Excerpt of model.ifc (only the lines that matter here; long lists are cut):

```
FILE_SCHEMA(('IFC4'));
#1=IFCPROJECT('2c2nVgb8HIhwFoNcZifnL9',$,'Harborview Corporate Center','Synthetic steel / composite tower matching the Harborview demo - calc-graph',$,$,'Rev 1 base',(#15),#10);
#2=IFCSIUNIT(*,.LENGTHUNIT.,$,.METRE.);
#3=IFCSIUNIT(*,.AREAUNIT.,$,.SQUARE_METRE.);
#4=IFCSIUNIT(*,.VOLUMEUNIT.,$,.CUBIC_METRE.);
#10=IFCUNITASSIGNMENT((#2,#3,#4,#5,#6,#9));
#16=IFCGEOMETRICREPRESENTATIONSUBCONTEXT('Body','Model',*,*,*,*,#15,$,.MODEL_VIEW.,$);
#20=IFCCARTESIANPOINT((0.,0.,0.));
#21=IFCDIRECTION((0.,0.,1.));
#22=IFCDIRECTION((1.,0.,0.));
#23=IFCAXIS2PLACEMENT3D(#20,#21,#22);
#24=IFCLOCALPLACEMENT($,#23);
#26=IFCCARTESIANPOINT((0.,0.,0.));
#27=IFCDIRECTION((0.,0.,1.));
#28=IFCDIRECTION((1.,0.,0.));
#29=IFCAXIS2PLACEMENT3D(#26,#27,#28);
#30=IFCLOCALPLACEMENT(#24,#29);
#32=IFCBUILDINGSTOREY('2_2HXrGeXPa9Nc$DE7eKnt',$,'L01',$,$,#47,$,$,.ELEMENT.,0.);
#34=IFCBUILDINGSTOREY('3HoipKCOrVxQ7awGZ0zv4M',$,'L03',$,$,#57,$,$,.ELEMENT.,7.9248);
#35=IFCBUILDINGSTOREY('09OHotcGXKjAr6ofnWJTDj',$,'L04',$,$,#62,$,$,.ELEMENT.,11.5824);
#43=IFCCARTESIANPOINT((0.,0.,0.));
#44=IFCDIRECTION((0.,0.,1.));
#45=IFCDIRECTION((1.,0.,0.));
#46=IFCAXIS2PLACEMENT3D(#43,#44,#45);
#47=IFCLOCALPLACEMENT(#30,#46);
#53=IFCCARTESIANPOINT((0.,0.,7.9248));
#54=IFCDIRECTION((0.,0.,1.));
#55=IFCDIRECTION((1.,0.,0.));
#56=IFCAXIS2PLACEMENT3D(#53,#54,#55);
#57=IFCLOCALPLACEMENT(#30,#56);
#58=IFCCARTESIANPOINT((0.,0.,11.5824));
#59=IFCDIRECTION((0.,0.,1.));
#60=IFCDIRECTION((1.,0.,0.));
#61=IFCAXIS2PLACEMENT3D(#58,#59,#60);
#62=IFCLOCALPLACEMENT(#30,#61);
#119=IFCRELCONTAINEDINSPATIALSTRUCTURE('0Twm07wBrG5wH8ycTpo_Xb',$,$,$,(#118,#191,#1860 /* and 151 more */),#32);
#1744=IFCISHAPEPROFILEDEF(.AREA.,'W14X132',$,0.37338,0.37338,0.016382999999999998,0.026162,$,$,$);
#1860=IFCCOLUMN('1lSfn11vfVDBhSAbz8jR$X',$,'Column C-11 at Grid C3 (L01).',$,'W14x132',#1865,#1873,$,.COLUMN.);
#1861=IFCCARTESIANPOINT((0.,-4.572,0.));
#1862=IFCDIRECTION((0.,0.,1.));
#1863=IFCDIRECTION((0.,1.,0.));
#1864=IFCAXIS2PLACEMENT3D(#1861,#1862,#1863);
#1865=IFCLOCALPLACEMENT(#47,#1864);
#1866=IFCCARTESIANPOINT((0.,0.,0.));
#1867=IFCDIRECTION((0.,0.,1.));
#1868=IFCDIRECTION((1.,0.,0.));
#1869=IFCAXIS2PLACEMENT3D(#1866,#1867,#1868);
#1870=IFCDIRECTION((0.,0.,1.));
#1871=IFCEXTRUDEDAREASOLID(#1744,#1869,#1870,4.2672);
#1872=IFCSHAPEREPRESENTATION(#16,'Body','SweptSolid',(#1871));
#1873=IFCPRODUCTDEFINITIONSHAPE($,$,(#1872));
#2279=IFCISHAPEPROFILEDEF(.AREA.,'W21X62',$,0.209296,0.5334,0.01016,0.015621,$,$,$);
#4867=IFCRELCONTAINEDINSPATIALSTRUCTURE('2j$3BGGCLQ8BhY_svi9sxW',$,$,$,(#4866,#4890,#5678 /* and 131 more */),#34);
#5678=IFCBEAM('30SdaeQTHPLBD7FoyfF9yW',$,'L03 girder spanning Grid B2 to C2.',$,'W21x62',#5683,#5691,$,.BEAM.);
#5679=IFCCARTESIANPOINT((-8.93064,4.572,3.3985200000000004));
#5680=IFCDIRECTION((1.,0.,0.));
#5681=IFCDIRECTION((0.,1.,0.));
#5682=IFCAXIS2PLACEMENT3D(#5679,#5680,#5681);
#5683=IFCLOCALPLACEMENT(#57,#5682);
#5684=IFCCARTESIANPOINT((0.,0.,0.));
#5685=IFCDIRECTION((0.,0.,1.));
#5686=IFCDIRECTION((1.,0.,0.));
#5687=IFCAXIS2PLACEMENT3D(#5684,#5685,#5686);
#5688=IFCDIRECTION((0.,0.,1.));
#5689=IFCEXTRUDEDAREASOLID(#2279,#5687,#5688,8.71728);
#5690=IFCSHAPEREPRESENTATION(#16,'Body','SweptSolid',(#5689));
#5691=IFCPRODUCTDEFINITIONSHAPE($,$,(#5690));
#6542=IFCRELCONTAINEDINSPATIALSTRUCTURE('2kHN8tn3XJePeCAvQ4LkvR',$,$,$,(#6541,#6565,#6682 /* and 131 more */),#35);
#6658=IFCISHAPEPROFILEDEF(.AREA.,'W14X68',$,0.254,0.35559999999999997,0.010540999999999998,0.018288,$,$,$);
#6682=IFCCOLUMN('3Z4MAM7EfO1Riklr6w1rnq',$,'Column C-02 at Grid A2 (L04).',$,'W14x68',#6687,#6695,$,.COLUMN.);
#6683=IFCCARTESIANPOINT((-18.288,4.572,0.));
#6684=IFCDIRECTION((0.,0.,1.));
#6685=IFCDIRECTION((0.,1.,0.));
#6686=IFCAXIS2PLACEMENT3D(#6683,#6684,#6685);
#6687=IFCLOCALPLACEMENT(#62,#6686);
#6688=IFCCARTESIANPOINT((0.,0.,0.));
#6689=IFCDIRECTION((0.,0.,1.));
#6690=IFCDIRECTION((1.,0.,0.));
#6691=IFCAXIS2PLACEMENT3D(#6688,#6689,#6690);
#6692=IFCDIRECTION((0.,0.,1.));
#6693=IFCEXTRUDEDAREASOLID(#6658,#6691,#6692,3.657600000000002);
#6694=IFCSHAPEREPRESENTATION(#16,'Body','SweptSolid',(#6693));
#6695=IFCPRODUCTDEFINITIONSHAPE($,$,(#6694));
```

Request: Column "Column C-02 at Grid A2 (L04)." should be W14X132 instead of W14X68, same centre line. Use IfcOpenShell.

```python
import ifcopenshell
import ifcopenshell.util.element
import ifcopenshell.util.representation

model = ifcopenshell.open("model.ifc")

member = model.by_id(6682)
source = next(p for p in model.by_type("IfcIShapeProfileDef") if p.ProfileName == "W14X132")

body = ifcopenshell.util.representation.get_representation(member, "Model", "Body")
solid = body.Items[0]
old_profile = solid.SweptArea

# Copy the section's sizes but keep this member's own profile position.
profile = ifcopenshell.util.element.copy(model, source)
profile.Position = old_profile.Position
solid.SweptArea = profile
if not model.get_total_inverses(old_profile):
    ifcopenshell.util.element.remove_deep2(model, old_profile)

print(solid.SweptArea)

model.write("model-out.ifc")
```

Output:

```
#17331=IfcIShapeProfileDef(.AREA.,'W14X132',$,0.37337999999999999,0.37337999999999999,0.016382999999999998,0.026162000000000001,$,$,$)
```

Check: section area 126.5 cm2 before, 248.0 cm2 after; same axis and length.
